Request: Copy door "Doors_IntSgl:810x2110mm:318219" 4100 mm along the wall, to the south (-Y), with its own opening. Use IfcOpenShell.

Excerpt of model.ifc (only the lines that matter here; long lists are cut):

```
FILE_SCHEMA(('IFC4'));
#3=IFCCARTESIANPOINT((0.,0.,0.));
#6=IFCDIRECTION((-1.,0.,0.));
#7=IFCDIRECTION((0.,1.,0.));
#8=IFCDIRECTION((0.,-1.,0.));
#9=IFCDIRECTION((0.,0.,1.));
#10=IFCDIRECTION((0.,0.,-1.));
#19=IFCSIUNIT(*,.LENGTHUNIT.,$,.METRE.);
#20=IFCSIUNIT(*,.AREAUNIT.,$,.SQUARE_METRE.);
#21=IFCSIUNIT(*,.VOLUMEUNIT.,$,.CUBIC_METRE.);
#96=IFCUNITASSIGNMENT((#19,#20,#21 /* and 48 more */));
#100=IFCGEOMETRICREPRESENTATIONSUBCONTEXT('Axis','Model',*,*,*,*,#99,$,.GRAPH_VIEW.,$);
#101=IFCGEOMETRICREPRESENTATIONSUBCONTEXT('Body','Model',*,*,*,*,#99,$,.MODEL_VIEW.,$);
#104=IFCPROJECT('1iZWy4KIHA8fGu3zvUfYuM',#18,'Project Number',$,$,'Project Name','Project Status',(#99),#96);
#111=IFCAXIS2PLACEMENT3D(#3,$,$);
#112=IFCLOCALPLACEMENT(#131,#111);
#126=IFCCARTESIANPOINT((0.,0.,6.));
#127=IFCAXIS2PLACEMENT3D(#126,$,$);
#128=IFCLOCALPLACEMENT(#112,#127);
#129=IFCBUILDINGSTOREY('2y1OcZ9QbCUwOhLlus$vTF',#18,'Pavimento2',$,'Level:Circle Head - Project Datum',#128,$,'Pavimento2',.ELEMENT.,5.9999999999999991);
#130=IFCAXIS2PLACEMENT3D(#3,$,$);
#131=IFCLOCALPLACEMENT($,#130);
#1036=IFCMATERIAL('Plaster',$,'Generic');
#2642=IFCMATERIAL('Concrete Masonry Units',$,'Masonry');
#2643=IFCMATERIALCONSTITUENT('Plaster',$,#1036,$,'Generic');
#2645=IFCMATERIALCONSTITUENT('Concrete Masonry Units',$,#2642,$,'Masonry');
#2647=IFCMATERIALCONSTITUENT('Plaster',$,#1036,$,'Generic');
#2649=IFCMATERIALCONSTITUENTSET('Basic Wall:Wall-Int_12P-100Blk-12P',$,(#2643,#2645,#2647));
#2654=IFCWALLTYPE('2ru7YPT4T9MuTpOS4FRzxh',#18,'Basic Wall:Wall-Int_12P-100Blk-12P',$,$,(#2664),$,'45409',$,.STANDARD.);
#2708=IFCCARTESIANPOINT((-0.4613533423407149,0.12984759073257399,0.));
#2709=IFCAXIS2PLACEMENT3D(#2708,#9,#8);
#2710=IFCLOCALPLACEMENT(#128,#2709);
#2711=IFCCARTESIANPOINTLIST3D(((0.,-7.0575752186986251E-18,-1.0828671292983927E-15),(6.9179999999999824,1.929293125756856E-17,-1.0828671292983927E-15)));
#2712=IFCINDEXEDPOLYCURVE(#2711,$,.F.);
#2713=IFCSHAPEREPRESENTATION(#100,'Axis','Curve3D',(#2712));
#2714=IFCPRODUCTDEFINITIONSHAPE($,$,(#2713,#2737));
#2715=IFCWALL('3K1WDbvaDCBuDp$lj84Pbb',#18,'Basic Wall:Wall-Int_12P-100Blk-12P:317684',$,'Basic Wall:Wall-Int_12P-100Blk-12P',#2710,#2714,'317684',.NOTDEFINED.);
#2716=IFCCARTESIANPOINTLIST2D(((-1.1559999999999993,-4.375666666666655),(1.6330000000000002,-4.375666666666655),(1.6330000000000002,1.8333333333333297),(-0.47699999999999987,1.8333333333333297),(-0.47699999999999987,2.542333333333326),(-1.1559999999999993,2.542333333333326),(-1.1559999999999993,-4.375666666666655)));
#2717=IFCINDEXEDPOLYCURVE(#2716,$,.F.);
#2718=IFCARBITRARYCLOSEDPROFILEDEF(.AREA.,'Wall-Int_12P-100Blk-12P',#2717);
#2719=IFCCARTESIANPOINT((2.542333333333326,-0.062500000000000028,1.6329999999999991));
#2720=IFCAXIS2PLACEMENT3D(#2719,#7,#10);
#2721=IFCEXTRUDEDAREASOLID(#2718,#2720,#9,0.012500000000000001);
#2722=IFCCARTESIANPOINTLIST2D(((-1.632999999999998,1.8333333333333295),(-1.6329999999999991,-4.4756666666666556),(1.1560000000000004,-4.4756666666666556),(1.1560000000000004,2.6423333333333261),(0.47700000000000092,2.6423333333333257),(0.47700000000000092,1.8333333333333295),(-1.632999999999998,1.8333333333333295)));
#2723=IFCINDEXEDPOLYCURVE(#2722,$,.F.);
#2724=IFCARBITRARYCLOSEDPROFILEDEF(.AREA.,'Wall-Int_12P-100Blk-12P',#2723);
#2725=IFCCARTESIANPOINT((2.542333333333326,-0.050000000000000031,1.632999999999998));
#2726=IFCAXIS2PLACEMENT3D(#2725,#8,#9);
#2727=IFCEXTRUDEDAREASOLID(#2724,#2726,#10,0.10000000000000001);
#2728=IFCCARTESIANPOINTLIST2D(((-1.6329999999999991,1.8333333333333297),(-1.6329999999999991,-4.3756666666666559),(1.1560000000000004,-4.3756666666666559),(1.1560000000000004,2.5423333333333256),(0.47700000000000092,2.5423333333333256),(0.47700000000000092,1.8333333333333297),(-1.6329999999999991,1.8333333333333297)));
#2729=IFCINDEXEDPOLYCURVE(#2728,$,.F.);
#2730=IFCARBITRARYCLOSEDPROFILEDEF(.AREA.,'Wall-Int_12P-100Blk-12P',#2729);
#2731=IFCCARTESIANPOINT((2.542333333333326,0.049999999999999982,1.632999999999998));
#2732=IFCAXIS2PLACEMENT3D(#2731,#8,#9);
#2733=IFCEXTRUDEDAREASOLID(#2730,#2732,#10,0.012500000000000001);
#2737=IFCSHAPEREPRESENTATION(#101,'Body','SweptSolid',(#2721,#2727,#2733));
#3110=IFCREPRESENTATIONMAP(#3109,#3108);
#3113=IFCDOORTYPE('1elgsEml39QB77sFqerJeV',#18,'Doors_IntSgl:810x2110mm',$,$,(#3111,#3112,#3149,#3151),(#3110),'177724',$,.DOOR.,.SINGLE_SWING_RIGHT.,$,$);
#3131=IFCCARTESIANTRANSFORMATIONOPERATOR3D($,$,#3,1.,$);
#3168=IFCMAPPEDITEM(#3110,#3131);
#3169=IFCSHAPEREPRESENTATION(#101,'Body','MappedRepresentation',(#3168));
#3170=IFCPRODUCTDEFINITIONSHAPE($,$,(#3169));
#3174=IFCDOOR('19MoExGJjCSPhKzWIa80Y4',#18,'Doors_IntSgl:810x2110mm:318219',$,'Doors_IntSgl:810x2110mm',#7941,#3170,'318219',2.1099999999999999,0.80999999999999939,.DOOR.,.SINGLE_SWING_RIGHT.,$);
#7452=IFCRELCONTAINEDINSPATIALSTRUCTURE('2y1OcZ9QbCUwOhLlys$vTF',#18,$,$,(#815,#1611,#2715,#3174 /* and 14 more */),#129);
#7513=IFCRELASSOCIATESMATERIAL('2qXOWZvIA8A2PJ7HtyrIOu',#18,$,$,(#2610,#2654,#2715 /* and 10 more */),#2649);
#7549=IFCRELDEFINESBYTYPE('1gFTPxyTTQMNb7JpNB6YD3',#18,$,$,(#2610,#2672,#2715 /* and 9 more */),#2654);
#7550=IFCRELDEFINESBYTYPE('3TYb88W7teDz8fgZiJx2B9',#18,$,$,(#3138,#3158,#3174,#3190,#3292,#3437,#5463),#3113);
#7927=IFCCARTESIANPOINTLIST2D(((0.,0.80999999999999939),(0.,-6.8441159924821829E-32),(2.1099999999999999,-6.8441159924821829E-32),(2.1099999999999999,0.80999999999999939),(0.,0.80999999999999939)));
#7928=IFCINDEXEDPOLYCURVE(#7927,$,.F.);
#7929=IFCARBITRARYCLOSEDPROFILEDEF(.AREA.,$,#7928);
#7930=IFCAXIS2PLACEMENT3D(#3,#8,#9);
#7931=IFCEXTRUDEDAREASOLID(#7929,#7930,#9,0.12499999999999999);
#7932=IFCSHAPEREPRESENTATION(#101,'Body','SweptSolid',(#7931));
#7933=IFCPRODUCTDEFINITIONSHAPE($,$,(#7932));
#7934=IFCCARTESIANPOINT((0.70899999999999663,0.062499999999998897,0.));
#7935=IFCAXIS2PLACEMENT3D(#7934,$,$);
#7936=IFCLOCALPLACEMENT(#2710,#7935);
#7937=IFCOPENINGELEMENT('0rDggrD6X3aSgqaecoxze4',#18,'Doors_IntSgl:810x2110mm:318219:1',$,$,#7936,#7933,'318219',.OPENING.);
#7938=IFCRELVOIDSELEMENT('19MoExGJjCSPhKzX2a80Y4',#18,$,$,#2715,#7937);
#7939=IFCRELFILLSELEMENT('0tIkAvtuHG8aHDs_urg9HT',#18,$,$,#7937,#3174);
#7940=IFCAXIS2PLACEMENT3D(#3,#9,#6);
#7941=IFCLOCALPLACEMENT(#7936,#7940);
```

```python
import ifcopenshell
import ifcopenshell.api.feature
import ifcopenshell.api.geometry
import ifcopenshell.api.root
import ifcopenshell.geom
import ifcopenshell.util.element
import ifcopenshell.util.placement
import ifcopenshell.util.shape

model = ifcopenshell.open("model.ifc")
settings = ifcopenshell.geom.settings()


def volume(element):
    """Net volume in cubic metres, openings subtracted."""
    shape = ifcopenshell.geom.create_shape(settings, element)
    return ifcopenshell.util.shape.get_volume(shape.geometry)


def reuse_history(source, copy):
    """copy_class also copies each property set's owner history, people and application; keep the originals."""
    for rel in copy.IsDefinedBy:
        if rel.is_a("IfcRelDefinesByProperties") and (history := rel.RelatingPropertyDefinition.OwnerHistory):
            rel.RelatingPropertyDefinition.OwnerHistory = source.OwnerHistory
            ifcopenshell.util.element.remove_deep2(model, history)


door = model.by_id(3174)
opening = door.FillsVoids[0].RelatingOpeningElement
wall = opening.VoidsElements[0].RelatingBuildingElement
before = volume(wall)
shift = ifcopenshell.util.placement.get_local_placement(wall.ObjectPlacement)[:3, 0] * 4.1

# copy_class copies the void relationship, type, container and properties, but no geometry.
new_opening = ifcopenshell.api.root.copy_class(model, product=opening)
new_opening.Representation = ifcopenshell.util.element.copy_deep(
    model, opening.Representation, exclude=["IfcGeometricRepresentationContext", "IfcRepresentationMap"]
)
new_opening.Name = "Doors_IntSgl:810x2110mm"
new_opening.Tag = None
new_door = ifcopenshell.api.root.copy_class(model, product=door)
new_door.Representation = ifcopenshell.util.element.copy_deep(
    model, door.Representation, exclude=["IfcGeometricRepresentationContext", "IfcRepresentationMap"]
)
new_door.Name = "Doors_IntSgl:810x2110mm"
new_door.Tag = None
reuse_history(door, new_door)
ifcopenshell.api.feature.add_filling(model, opening=new_opening, element=new_door)

for old, new in ((opening, new_opening), (door, new_door)):
    matrix = ifcopenshell.util.placement.get_local_placement(old.ObjectPlacement)
    matrix[:3, 3] += shift
    ifcopenshell.api.geometry.edit_object_placement(model, product=new, matrix=matrix, is_si=False)

after = volume(wall)

print(f"wall volume {before:.3f} -> {after:.3f} m3")

model.write("model_updated.ifc")
```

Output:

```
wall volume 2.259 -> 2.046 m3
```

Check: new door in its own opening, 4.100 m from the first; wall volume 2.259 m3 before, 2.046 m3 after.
